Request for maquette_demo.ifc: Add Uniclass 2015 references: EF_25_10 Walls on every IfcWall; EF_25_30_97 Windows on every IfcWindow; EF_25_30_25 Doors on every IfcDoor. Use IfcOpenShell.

First a look at what the model holds.

```python
import ifcopenshell

model = ifcopenshell.open("maquette_demo.ifc")
print(model.schema)
print("classifications:", [c.Name for c in model.by_type("IfcClassification")])
for ifc_class in ("IfcDoor", "IfcRoof", "IfcStair", "IfcWall", "IfcWindow"):
    print(ifc_class, len(model.by_type(ifc_class)))
```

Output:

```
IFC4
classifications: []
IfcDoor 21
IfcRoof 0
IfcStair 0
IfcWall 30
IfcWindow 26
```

```python
import ifcopenshell
import ifcopenshell.api.classification

model = ifcopenshell.open("maquette_demo.ifc")

system = ifcopenshell.api.classification.add_classification(model, classification="Uniclass 2015")

codes = {
    "IfcWall": ("EF_25_10", "Walls"),
    "IfcWindow": ("EF_25_30_97", "Windows"),
    "IfcDoor": ("EF_25_30_25", "Doors"),
}
for ifc_class, (code, name) in codes.items():
    products = model.by_type(ifc_class)
    ifcopenshell.api.classification.add_reference(
        model, products=products, classification=system, identification=code, name=name
    )
    print(code, len(products))

model.write("maquette_demo-out.ifc")
```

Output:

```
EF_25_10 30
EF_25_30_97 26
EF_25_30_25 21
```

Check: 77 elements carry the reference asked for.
